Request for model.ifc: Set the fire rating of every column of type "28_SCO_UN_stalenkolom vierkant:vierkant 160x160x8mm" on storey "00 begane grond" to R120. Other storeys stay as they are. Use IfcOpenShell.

First a look at what the model holds.

```python
import ifcopenshell
import ifcopenshell.util.element

model = ifcopenshell.open("model.ifc")
print(model.schema)
storey = next(s for s in model.by_type("IfcBuildingStorey") if s.Name == "00 begane grond")
columns = [e for e in ifcopenshell.util.element.get_decomposition(storey) if e.is_a("IfcColumn")]
seen = {}
for e in columns:
    element_type = ifcopenshell.util.element.get_type(e)
    key = (element_type.Name if element_type != e and element_type else None, ifcopenshell.util.element.get_pset(e, "Pset_ColumnCommon", "FireRating"))
    seen[key] = seen.get(key, 0) + 1
for (name, value), count in sorted(seen.items(), key=str):
    print(count, "x", name, "|", value)
```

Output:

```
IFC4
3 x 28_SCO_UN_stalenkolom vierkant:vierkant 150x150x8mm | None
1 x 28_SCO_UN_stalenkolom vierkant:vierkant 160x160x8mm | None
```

```python
import ifcopenshell
import ifcopenshell.api.pset
import ifcopenshell.util.element

model = ifcopenshell.open("model.ifc")

storey = next(s for s in model.by_type("IfcBuildingStorey") if s.Name == "00 begane grond")
columns = [e for e in ifcopenshell.util.element.get_decomposition(storey) if e.is_a("IfcColumn")]

count = 0
for e in columns:
    element_type = ifcopenshell.util.element.get_type(e)
    if element_type in (None, e) or element_type.Name != "28_SCO_UN_stalenkolom vierkant:vierkant 160x160x8mm":
        continue
    # add_pset returns the element's existing set when there is one.
    pset = ifcopenshell.api.pset.add_pset(model, product=e, name="Pset_ColumnCommon")
    ifcopenshell.api.pset.edit_pset(model, pset=pset, properties={"FireRating": "R120"})
    count += 1

print(count, "columns updated")

model.write("model_edited.ifc")
```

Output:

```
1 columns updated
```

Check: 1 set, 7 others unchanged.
